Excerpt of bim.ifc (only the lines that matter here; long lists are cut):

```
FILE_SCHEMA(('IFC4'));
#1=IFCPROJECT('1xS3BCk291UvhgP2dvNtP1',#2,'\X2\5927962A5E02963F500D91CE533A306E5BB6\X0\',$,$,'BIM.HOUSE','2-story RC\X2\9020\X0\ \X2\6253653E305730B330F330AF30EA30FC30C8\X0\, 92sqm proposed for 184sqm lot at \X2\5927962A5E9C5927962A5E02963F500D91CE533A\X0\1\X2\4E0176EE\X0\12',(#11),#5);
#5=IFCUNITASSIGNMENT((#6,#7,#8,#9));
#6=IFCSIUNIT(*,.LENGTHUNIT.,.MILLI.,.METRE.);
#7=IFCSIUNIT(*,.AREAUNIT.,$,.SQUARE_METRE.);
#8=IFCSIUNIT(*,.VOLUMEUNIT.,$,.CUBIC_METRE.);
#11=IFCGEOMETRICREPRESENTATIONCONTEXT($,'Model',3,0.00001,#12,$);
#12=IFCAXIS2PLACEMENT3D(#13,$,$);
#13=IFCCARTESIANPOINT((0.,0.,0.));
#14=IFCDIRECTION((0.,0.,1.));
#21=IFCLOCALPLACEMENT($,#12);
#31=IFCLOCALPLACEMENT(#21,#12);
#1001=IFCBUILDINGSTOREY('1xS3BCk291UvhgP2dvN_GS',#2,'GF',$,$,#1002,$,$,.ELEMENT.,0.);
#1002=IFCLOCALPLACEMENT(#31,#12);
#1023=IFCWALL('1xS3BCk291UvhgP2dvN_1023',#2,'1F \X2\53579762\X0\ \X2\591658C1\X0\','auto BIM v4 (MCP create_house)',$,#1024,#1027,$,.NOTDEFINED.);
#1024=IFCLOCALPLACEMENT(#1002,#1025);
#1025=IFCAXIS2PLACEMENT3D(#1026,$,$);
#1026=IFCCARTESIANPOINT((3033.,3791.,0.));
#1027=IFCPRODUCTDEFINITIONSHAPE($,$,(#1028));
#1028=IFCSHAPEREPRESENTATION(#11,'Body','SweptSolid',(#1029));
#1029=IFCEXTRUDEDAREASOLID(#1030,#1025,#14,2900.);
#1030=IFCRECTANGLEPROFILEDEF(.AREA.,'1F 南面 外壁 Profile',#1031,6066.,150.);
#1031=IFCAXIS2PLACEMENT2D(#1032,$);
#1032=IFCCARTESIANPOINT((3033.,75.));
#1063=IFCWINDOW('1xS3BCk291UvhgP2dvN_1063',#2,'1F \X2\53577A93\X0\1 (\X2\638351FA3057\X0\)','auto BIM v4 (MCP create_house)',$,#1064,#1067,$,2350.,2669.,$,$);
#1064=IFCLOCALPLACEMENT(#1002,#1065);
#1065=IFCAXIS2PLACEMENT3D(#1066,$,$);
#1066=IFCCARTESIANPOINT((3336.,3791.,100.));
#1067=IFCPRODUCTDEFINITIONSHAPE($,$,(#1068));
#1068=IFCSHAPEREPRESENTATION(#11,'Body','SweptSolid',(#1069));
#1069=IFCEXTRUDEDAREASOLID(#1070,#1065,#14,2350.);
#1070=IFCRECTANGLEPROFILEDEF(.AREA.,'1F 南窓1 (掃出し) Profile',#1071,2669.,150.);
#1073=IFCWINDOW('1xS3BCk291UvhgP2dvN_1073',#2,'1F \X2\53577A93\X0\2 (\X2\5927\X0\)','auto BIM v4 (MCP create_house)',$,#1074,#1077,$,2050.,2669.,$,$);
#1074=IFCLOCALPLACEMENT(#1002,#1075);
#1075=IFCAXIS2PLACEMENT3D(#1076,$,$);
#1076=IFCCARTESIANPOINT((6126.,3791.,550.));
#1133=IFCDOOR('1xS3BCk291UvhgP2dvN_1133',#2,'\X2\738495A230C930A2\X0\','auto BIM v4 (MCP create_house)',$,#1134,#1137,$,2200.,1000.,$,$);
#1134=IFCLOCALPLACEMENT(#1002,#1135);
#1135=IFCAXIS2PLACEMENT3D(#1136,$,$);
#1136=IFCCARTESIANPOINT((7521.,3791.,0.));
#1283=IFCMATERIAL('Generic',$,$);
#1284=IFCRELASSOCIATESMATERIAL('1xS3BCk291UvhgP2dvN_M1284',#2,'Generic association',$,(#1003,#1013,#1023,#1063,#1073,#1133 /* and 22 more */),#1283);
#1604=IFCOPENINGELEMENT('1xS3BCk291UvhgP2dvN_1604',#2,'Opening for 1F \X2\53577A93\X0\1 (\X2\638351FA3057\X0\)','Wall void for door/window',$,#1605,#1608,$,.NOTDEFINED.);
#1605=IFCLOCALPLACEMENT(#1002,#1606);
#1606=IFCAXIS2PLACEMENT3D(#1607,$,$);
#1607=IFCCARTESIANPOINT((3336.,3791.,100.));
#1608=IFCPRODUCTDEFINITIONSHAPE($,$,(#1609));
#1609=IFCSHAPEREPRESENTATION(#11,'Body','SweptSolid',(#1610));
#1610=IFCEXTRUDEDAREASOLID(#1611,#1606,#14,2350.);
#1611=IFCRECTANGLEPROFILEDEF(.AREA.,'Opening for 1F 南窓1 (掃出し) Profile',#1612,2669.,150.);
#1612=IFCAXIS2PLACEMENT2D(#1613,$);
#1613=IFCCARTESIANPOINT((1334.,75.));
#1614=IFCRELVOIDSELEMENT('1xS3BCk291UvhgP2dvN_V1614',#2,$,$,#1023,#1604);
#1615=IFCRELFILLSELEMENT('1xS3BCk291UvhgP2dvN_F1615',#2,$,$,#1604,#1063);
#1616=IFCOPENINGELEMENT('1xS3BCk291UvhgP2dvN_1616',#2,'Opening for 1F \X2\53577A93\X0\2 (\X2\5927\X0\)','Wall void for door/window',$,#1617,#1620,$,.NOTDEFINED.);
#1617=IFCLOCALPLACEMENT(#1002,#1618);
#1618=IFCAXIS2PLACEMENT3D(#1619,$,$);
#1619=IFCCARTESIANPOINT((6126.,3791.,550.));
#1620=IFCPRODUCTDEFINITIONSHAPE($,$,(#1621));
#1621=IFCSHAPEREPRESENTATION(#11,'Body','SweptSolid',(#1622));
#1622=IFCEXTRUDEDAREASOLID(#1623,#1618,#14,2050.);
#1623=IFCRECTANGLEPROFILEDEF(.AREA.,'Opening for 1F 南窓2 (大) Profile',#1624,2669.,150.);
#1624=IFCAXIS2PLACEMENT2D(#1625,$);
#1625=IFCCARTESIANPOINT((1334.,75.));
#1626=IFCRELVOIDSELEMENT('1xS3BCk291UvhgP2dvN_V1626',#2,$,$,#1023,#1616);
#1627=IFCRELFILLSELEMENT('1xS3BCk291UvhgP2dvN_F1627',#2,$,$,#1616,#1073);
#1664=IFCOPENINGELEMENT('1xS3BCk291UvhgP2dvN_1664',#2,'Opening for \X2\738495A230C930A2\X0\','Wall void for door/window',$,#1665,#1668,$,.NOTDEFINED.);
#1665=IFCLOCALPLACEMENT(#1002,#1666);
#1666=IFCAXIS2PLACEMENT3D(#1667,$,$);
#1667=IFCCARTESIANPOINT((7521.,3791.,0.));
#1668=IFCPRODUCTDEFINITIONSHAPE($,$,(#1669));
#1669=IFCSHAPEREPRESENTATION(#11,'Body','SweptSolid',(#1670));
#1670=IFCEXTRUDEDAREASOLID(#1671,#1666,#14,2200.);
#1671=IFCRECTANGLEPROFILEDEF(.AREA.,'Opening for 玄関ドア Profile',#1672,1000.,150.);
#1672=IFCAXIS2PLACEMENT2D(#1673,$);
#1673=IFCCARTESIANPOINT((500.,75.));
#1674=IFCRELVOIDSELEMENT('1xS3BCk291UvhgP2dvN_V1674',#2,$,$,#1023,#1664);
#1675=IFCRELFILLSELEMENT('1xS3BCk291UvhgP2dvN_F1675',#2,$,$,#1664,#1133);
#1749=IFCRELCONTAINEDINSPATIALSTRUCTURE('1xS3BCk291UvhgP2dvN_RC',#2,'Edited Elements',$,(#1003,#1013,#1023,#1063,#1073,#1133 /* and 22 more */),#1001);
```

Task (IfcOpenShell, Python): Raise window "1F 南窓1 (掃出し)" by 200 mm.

```python
import numpy as np
import ifcopenshell
import ifcopenshell.api.geometry
import ifcopenshell.util.placement
import ifcopenshell.util.unit

model = ifcopenshell.open("bim.ifc")
unit_scale = ifcopenshell.util.unit.calculate_unit_scale(model)

window = model.by_guid("1xS3BCk291UvhgP2dvN_1063")
opening = window.FillsVoids[0].RelatingOpeningElement
dz = 200.0

shift = np.array([0.0, 0.0, dz])
# The window is not placed relative to its opening, so move both.
for product in (opening, window):
    matrix = ifcopenshell.util.placement.get_local_placement(product.ObjectPlacement)
    matrix[:3, 3] += shift
    ifcopenshell.api.geometry.edit_object_placement(model, product=product, matrix=matrix, is_si=False)

print(f"moved by {dz * unit_scale:+.3f} m")

model.write("bim_rev.ifc")
```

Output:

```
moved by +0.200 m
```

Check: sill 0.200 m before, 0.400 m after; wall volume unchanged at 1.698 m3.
